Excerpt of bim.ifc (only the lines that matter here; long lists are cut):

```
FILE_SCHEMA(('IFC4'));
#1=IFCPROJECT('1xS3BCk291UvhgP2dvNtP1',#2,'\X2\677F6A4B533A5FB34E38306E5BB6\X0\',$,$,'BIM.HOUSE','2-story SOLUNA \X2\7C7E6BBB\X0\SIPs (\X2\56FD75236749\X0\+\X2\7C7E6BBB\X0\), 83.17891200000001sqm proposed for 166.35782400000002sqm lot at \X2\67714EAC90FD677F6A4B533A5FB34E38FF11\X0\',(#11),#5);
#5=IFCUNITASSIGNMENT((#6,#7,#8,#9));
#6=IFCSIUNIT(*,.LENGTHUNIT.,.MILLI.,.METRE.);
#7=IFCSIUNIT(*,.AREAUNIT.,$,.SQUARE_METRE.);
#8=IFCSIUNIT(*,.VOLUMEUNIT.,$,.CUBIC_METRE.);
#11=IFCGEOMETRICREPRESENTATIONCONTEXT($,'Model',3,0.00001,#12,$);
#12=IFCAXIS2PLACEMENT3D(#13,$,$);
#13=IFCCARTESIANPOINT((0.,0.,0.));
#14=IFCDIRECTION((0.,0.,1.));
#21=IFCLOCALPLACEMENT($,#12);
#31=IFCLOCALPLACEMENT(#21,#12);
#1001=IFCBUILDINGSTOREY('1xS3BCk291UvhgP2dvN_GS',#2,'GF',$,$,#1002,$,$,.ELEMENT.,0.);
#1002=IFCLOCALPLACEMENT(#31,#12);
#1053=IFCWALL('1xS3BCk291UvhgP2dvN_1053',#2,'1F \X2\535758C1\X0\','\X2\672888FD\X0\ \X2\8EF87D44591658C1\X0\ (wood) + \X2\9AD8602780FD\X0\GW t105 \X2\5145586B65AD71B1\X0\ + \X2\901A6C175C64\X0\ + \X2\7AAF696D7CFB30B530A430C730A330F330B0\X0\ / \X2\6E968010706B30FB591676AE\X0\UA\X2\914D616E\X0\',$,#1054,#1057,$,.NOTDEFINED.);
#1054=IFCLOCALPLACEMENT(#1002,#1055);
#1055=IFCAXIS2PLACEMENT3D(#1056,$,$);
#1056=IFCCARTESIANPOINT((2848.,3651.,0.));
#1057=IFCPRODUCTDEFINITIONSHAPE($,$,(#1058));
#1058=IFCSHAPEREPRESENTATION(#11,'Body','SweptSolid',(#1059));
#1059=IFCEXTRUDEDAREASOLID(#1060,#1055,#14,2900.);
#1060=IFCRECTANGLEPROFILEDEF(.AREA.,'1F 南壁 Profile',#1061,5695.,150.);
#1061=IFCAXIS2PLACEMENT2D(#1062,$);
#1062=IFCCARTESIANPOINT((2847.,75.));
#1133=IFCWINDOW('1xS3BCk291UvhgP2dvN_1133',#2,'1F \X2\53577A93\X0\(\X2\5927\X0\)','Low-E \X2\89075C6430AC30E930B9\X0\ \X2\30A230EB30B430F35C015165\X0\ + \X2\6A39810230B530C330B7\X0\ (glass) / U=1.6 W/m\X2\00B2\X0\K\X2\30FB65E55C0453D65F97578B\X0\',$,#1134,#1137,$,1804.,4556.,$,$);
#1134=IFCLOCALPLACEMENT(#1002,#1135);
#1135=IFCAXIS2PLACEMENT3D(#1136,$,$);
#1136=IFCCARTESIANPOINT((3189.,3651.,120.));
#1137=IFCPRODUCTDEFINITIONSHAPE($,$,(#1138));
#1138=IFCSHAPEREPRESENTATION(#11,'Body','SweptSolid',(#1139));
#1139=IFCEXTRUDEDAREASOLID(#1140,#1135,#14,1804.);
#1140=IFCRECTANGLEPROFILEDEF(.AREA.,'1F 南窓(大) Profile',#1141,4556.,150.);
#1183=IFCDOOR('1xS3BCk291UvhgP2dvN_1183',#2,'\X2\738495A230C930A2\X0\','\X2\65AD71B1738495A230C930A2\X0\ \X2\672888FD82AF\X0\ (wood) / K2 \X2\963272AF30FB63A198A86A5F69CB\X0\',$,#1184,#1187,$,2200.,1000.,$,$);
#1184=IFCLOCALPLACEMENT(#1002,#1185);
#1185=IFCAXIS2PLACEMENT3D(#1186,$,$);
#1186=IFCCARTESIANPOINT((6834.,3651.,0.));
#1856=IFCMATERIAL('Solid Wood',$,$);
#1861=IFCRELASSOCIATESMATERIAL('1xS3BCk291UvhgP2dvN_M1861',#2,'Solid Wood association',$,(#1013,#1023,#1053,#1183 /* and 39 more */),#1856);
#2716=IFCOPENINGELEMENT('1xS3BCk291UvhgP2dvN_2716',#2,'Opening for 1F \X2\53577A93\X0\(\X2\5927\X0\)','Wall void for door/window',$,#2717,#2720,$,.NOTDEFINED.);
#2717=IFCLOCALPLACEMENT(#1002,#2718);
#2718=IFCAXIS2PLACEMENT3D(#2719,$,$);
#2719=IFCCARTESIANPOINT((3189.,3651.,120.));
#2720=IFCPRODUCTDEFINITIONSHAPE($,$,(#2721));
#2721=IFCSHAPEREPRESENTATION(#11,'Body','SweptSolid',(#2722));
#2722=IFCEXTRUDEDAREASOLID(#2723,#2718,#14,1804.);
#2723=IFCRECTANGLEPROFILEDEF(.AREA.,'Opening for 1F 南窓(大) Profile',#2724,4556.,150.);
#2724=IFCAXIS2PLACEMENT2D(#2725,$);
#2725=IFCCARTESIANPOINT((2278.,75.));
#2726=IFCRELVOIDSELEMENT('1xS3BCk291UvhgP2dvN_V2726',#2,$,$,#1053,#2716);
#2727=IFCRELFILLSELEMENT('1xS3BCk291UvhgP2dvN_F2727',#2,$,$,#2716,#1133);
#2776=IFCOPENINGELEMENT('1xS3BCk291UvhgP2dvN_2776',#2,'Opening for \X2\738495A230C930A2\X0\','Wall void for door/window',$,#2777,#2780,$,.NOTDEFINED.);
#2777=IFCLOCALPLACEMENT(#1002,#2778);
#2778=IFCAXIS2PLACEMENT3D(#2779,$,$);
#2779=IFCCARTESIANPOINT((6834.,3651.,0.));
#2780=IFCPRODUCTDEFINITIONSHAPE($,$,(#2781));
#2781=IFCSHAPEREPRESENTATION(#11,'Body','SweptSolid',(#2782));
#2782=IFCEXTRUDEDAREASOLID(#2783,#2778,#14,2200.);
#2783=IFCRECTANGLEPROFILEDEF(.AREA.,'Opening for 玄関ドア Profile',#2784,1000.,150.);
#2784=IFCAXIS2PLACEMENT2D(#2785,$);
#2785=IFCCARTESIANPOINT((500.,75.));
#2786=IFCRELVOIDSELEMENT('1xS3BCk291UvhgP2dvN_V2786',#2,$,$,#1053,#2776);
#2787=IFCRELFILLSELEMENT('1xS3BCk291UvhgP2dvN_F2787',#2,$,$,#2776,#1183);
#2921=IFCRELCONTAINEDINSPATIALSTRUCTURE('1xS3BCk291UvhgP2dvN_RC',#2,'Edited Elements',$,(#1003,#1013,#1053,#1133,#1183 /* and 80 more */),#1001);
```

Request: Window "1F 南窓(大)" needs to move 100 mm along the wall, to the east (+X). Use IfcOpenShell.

```python
import ifcopenshell
import ifcopenshell.api.geometry
import ifcopenshell.util.placement
import ifcopenshell.util.unit

model = ifcopenshell.open("bim.ifc")
unit_scale = ifcopenshell.util.unit.calculate_unit_scale(model)

window = model.by_guid("1xS3BCk291UvhgP2dvN_1133")
opening = window.FillsVoids[0].RelatingOpeningElement
wall = opening.VoidsElements[0].RelatingBuildingElement

wall_matrix = ifcopenshell.util.placement.get_local_placement(wall.ObjectPlacement)
shift = wall_matrix[:3, 0] * 0.1 / unit_scale
before = ifcopenshell.util.placement.get_local_placement(window.ObjectPlacement)[:3, 3].copy()

# The window is not placed relative to its opening, so move both.
for product in (opening, window):
    matrix = ifcopenshell.util.placement.get_local_placement(product.ObjectPlacement)
    matrix[:3, 3] += shift
    ifcopenshell.api.geometry.edit_object_placement(model, product=product, matrix=matrix, is_si=False)

after = ifcopenshell.util.placement.get_local_placement(window.ObjectPlacement)[:3, 3]
print("window moved by", (after - before).round(3) + 0.0)

model.write("bim_edited.ifc")
```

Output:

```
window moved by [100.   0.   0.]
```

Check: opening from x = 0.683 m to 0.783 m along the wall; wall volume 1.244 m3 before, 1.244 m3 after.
